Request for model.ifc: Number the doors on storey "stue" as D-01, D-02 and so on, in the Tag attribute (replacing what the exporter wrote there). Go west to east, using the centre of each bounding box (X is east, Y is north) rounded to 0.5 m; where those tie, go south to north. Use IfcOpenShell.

First a look at what the model holds.

```python
import ifcopenshell
import ifcopenshell.util.element
import ifcopenshell.util.placement

model = ifcopenshell.open("model.ifc")
print(model.schema)
storey = next(s for s in model.by_type("IfcBuildingStorey") if s.Name == "stue")
doors = [e for e in ifcopenshell.util.element.get_decomposition(storey) if e.is_a("IfcDoor")]
for e in sorted(doors, key=lambda e: e.id()):
    origin = ifcopenshell.util.placement.get_local_placement(e.ObjectPlacement)[:3, 3]
    print(e.id(), e.Tag, e.Name, origin.round(2) + 0.0, sep=" | ")
```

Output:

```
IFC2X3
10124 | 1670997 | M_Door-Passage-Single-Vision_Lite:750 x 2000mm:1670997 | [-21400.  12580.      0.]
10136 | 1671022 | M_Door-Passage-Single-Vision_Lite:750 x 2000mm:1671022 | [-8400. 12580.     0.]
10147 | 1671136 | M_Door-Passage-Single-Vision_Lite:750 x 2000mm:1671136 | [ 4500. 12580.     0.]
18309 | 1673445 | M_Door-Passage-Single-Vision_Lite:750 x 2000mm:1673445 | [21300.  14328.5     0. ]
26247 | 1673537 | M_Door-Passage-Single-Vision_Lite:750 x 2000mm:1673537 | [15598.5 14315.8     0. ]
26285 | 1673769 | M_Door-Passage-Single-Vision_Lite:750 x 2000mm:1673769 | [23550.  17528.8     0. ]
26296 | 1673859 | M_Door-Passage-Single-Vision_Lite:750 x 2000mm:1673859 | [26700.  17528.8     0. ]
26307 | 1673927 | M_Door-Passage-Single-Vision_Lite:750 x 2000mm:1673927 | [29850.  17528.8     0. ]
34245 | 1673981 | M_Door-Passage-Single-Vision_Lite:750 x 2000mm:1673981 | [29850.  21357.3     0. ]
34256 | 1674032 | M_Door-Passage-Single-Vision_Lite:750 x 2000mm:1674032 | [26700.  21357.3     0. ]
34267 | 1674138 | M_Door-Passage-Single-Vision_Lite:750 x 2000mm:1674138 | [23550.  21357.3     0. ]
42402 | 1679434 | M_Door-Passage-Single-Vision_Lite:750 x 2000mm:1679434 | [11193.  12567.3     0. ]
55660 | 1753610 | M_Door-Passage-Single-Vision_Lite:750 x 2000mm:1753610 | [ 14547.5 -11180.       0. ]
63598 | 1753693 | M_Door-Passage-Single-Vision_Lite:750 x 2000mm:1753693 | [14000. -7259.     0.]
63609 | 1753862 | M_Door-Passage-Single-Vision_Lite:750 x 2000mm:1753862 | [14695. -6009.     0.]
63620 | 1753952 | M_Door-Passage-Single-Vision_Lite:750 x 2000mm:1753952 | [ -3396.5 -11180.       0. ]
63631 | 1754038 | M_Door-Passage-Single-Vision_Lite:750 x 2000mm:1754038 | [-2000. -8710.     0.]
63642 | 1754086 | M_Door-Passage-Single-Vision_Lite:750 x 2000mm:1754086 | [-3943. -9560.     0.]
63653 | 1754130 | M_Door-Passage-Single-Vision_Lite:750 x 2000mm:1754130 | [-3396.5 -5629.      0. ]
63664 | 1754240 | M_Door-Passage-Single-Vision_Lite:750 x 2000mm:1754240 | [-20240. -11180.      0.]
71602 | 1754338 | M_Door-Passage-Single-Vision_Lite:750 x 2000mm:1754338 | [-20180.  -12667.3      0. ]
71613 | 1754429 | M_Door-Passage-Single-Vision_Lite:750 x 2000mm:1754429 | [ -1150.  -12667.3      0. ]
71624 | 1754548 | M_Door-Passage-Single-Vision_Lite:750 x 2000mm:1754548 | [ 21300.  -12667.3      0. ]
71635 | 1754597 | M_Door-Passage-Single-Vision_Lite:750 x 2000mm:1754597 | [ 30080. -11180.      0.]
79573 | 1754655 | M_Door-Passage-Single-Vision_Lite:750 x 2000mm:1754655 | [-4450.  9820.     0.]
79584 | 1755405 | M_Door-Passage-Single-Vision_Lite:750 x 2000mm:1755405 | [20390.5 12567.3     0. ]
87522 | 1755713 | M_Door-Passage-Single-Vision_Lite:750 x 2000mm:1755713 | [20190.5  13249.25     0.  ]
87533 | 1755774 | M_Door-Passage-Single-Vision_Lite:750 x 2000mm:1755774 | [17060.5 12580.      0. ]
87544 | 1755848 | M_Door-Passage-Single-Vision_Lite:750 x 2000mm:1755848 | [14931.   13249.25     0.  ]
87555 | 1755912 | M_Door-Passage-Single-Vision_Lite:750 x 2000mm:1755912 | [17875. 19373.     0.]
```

```python
import ifcopenshell
import ifcopenshell.geom
import ifcopenshell.util.element
import ifcopenshell.util.shape

model = ifcopenshell.open("model.ifc")
settings = ifcopenshell.geom.settings()
settings.set("use-world-coords", True)


def centre(element):
    shape = ifcopenshell.geom.create_shape(settings, element)
    return ifcopenshell.util.shape.get_bbox_centroid(shape.geometry)


storey = next(s for s in model.by_type("IfcBuildingStorey") if s.Name == "stue")
doors = [e for e in ifcopenshell.util.element.get_decomposition(storey) if e.is_a("IfcDoor")]

# Insertion points can sit at a corner or the storey origin, so sort by the geometry (in metres).
centres = {e: centre(e) for e in doors}
doors.sort(key=lambda e: (round(centres[e][0] / 0.5), centres[e][1]))

for i, e in enumerate(doors, start=1):
    number = f"D-{i:02d}"
    e.Tag = number
    print(e.id(), number)

model.write("model_v2.ifc")
```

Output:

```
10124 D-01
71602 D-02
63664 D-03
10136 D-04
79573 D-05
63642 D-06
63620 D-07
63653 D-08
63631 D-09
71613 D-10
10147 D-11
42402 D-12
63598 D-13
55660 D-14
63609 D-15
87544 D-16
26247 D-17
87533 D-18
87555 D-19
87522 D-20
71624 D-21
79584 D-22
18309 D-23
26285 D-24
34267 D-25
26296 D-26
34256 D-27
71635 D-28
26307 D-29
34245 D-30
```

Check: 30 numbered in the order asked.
